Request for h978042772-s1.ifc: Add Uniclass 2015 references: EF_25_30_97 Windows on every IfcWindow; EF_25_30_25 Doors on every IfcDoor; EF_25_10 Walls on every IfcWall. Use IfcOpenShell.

First a look at what the model holds.

```python
import ifcopenshell

model = ifcopenshell.open("h978042772-s1.ifc")
print(model.schema)
print("classifications:", [c.Name for c in model.by_type("IfcClassification")])
for ifc_class in ("IfcDoor", "IfcRoof", "IfcStair", "IfcWall", "IfcWindow"):
    print(ifc_class, len(model.by_type(ifc_class)))
```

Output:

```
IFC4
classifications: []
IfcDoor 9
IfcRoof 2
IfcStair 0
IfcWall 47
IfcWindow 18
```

```python
import ifcopenshell
import ifcopenshell.api.classification

model = ifcopenshell.open("h978042772-s1.ifc")

system = ifcopenshell.api.classification.add_classification(model, classification="Uniclass 2015")

codes = {
    "IfcWindow": ("EF_25_30_97", "Windows"),
    "IfcDoor": ("EF_25_30_25", "Doors"),
    "IfcWall": ("EF_25_10", "Walls"),
}
for ifc_class, (code, name) in codes.items():
    products = model.by_type(ifc_class)
    ifcopenshell.api.classification.add_reference(
        model, products=products, classification=system, identification=code, name=name
    )
    print(code, len(products))

model.write("h978042772-s1_edited.ifc")
```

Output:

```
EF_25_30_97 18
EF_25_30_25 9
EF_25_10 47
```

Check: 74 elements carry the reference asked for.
